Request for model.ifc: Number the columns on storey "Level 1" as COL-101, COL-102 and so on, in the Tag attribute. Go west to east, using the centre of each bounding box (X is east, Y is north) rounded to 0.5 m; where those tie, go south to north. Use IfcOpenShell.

First a look at what the model holds.

```python
import ifcopenshell
import ifcopenshell.util.element
import ifcopenshell.util.placement

model = ifcopenshell.open("model.ifc")
print(model.schema)
storey = next(s for s in model.by_type("IfcBuildingStorey") if s.Name == "Level 1")
columns = [e for e in ifcopenshell.util.element.get_decomposition(storey) if e.is_a("IfcColumn")]
for e in sorted(columns, key=lambda e: e.id()):
    origin = ifcopenshell.util.placement.get_local_placement(e.ObjectPlacement)[:3, 3]
    print(e.id(), e.Tag, e.Name, origin.round(2) + 0.0, sep=" | ")
```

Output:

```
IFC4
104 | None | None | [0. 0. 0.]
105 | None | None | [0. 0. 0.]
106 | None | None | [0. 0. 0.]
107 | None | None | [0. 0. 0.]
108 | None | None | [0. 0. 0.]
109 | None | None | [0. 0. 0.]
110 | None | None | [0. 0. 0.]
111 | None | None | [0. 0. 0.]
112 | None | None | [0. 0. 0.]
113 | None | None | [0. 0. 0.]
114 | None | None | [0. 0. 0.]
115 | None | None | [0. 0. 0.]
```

```python
import ifcopenshell
import ifcopenshell.geom
import ifcopenshell.util.element
import ifcopenshell.util.shape

model = ifcopenshell.open("model.ifc")
settings = ifcopenshell.geom.settings()
settings.set("use-world-coords", True)


def centre(element):
    shape = ifcopenshell.geom.create_shape(settings, element)
    return ifcopenshell.util.shape.get_bbox_centroid(shape.geometry)


storey = next(s for s in model.by_type("IfcBuildingStorey") if s.Name == "Level 1")
columns = [e for e in ifcopenshell.util.element.get_decomposition(storey) if e.is_a("IfcColumn")]

# Insertion points can sit at a corner or the storey origin, so sort by the geometry (in metres).
centres = {e: centre(e) for e in columns}
columns.sort(key=lambda e: (round(centres[e][0] / 0.5), centres[e][1]))

for i, e in enumerate(columns, start=1):
    number = f"COL-1{i:02d}"
    e.Tag = number
    print(e.id(), number)

model.write("model_updated.ifc")
```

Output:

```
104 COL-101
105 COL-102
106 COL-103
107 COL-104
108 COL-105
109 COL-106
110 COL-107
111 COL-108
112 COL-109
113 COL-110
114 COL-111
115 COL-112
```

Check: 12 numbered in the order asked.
